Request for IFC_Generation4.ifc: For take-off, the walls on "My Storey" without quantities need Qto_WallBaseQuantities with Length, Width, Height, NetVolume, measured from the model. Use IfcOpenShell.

First a look at what the model holds.

```python
import ifcopenshell
import ifcopenshell.util.element
import ifcopenshell.util.unit

model = ifcopenshell.open("IFC_Generation4.ifc")
print(model.schema)
for unit_type in ("LENGTHUNIT", "AREAUNIT", "VOLUMEUNIT"):
    print(unit_type, ifcopenshell.util.unit.calculate_unit_scale(model, unit_type))
storey = next(s for s in model.by_type("IfcBuildingStorey") if s.Name == "My Storey")
walls = [e for e in ifcopenshell.util.element.get_decomposition(storey) if e.is_a("IfcWall")]
for e in sorted(walls, key=lambda e: e.id()):
    print(e.id(), e.is_a(), e.Name, list(ifcopenshell.util.element.get_psets(e, qtos_only=True)), sep=" | ")
```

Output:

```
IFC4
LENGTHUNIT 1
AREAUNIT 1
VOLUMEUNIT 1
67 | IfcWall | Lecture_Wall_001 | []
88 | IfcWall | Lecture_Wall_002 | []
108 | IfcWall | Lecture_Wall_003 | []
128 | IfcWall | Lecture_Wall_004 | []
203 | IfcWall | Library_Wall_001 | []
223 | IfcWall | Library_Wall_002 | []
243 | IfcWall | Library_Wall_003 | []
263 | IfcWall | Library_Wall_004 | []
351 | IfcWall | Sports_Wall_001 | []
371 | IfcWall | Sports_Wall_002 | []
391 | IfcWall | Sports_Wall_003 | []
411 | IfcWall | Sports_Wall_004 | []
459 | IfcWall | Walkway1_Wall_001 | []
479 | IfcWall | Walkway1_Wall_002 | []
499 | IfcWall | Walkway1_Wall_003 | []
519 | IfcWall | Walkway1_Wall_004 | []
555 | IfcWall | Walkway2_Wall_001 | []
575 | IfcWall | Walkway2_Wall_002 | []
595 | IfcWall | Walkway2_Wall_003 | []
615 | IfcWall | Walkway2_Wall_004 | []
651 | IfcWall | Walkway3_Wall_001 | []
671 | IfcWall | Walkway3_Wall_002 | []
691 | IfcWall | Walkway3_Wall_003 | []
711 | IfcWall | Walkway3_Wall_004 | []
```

```python
import ifcopenshell
import ifcopenshell.api.pset
import ifcopenshell.geom
import ifcopenshell.util.element
import ifcopenshell.util.shape
import ifcopenshell.util.unit

model = ifcopenshell.open("IFC_Generation4.ifc")
unit_scale = ifcopenshell.util.unit.calculate_unit_scale(model)
volume_scale = ifcopenshell.util.unit.calculate_unit_scale(model, "VOLUMEUNIT")
settings = ifcopenshell.geom.settings()

storey = next(s for s in model.by_type("IfcBuildingStorey") if s.Name == "My Storey")
walls = [e for e in ifcopenshell.util.element.get_decomposition(storey) if e.is_a("IfcWall")]

for e in sorted(walls, key=lambda e: e.id()):
    if ifcopenshell.util.element.get_psets(e, qtos_only=True, should_inherit=False):
        continue
    # Geometry comes back in metres, in the element's own axes.
    shape = ifcopenshell.geom.create_shape(settings, e)
    values = {
        "Length": ifcopenshell.util.shape.get_x(shape.geometry) / unit_scale,
        "Width": ifcopenshell.util.shape.get_y(shape.geometry) / unit_scale,
        "Height": ifcopenshell.util.shape.get_z(shape.geometry) / unit_scale,
        "NetVolume": ifcopenshell.util.shape.get_volume(shape.geometry) / volume_scale,
    }
    qto = ifcopenshell.api.pset.add_qto(model, product=e, name="Qto_WallBaseQuantities")
    ifcopenshell.api.pset.edit_qto(model, qto=qto, properties=values)
    print(e.id(), {k: round(v, 3) for k, v in values.items()})

model.write("IFC_Generation4_v2.ifc")
```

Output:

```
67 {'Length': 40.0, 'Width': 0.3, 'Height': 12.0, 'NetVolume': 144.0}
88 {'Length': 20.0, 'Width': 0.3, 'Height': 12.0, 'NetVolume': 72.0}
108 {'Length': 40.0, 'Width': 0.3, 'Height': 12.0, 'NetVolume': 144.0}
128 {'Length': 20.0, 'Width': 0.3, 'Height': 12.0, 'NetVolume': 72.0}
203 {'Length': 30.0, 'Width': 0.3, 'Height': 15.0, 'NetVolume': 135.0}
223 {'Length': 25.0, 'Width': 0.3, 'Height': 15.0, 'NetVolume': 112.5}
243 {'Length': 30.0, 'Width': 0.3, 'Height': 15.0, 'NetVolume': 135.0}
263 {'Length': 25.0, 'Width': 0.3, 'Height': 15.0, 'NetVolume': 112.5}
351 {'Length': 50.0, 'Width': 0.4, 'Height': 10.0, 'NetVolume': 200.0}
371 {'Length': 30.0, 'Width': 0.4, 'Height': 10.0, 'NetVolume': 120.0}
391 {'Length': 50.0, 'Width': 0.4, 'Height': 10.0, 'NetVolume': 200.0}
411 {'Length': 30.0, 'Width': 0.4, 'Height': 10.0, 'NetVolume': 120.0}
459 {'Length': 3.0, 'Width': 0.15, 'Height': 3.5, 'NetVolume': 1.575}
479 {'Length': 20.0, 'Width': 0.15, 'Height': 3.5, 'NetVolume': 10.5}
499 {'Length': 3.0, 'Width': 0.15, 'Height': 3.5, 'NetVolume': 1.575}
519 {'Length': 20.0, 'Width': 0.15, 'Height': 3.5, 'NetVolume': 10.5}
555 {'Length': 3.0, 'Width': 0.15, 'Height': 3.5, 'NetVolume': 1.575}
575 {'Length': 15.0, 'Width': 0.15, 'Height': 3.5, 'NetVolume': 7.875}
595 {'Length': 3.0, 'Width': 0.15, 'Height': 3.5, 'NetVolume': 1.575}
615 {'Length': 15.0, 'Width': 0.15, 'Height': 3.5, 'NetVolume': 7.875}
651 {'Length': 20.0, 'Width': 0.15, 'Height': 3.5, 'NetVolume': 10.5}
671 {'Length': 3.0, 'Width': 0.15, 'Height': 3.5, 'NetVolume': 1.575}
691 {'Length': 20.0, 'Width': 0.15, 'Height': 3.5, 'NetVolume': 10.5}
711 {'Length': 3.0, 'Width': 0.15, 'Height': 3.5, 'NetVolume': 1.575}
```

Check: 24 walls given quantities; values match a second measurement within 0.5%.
